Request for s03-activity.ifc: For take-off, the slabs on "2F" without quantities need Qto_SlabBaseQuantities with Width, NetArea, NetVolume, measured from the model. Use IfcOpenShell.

First a look at what the model holds.

```python
import ifcopenshell
import ifcopenshell.util.element
import ifcopenshell.util.unit

model = ifcopenshell.open("s03-activity.ifc")
print(model.schema)
for unit_type in ("LENGTHUNIT", "AREAUNIT", "VOLUMEUNIT"):
    print(unit_type, ifcopenshell.util.unit.calculate_unit_scale(model, unit_type))
storey = next(s for s in model.by_type("IfcBuildingStorey") if s.Name == "2F")
slabs = [e for e in ifcopenshell.util.element.get_decomposition(storey) if e.is_a("IfcSlab")]
for e in sorted(slabs, key=lambda e: e.id()):
    print(e.id(), e.is_a(), e.Name, list(ifcopenshell.util.element.get_psets(e, qtos_only=True)), sep=" | ")
```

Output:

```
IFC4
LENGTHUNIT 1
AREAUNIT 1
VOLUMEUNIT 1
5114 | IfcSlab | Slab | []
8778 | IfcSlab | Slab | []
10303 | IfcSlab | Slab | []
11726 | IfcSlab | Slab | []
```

```python
import ifcopenshell
import ifcopenshell.api.pset
import ifcopenshell.geom
import ifcopenshell.util.element
import ifcopenshell.util.shape
import ifcopenshell.util.unit

model = ifcopenshell.open("s03-activity.ifc")
unit_scale = ifcopenshell.util.unit.calculate_unit_scale(model)
area_scale = ifcopenshell.util.unit.calculate_unit_scale(model, "AREAUNIT")
volume_scale = ifcopenshell.util.unit.calculate_unit_scale(model, "VOLUMEUNIT")
settings = ifcopenshell.geom.settings()

storey = next(s for s in model.by_type("IfcBuildingStorey") if s.Name == "2F")
slabs = [e for e in ifcopenshell.util.element.get_decomposition(storey) if e.is_a("IfcSlab")]

for e in sorted(slabs, key=lambda e: e.id()):
    if ifcopenshell.util.element.get_psets(e, qtos_only=True, should_inherit=False):
        continue
    # Geometry comes back in metres, in the element's own axes.
    shape = ifcopenshell.geom.create_shape(settings, e)
    values = {
        "Width": ifcopenshell.util.shape.get_z(shape.geometry) / unit_scale,
        "NetArea": ifcopenshell.util.shape.get_footprint_area(shape.geometry) / area_scale,
        "NetVolume": ifcopenshell.util.shape.get_volume(shape.geometry) / volume_scale,
    }
    qto = ifcopenshell.api.pset.add_qto(model, product=e, name="Qto_SlabBaseQuantities")
    ifcopenshell.api.pset.edit_qto(model, qto=qto, properties=values)
    print(e.id(), {k: round(v, 3) for k, v in values.items()})

model.write("s03-activity_rev.ifc")
```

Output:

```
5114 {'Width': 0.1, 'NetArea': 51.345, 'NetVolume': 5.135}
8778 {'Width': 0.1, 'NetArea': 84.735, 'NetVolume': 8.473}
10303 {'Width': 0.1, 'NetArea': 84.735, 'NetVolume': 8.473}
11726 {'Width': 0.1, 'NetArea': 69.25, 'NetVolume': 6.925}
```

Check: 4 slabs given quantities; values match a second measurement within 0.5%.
